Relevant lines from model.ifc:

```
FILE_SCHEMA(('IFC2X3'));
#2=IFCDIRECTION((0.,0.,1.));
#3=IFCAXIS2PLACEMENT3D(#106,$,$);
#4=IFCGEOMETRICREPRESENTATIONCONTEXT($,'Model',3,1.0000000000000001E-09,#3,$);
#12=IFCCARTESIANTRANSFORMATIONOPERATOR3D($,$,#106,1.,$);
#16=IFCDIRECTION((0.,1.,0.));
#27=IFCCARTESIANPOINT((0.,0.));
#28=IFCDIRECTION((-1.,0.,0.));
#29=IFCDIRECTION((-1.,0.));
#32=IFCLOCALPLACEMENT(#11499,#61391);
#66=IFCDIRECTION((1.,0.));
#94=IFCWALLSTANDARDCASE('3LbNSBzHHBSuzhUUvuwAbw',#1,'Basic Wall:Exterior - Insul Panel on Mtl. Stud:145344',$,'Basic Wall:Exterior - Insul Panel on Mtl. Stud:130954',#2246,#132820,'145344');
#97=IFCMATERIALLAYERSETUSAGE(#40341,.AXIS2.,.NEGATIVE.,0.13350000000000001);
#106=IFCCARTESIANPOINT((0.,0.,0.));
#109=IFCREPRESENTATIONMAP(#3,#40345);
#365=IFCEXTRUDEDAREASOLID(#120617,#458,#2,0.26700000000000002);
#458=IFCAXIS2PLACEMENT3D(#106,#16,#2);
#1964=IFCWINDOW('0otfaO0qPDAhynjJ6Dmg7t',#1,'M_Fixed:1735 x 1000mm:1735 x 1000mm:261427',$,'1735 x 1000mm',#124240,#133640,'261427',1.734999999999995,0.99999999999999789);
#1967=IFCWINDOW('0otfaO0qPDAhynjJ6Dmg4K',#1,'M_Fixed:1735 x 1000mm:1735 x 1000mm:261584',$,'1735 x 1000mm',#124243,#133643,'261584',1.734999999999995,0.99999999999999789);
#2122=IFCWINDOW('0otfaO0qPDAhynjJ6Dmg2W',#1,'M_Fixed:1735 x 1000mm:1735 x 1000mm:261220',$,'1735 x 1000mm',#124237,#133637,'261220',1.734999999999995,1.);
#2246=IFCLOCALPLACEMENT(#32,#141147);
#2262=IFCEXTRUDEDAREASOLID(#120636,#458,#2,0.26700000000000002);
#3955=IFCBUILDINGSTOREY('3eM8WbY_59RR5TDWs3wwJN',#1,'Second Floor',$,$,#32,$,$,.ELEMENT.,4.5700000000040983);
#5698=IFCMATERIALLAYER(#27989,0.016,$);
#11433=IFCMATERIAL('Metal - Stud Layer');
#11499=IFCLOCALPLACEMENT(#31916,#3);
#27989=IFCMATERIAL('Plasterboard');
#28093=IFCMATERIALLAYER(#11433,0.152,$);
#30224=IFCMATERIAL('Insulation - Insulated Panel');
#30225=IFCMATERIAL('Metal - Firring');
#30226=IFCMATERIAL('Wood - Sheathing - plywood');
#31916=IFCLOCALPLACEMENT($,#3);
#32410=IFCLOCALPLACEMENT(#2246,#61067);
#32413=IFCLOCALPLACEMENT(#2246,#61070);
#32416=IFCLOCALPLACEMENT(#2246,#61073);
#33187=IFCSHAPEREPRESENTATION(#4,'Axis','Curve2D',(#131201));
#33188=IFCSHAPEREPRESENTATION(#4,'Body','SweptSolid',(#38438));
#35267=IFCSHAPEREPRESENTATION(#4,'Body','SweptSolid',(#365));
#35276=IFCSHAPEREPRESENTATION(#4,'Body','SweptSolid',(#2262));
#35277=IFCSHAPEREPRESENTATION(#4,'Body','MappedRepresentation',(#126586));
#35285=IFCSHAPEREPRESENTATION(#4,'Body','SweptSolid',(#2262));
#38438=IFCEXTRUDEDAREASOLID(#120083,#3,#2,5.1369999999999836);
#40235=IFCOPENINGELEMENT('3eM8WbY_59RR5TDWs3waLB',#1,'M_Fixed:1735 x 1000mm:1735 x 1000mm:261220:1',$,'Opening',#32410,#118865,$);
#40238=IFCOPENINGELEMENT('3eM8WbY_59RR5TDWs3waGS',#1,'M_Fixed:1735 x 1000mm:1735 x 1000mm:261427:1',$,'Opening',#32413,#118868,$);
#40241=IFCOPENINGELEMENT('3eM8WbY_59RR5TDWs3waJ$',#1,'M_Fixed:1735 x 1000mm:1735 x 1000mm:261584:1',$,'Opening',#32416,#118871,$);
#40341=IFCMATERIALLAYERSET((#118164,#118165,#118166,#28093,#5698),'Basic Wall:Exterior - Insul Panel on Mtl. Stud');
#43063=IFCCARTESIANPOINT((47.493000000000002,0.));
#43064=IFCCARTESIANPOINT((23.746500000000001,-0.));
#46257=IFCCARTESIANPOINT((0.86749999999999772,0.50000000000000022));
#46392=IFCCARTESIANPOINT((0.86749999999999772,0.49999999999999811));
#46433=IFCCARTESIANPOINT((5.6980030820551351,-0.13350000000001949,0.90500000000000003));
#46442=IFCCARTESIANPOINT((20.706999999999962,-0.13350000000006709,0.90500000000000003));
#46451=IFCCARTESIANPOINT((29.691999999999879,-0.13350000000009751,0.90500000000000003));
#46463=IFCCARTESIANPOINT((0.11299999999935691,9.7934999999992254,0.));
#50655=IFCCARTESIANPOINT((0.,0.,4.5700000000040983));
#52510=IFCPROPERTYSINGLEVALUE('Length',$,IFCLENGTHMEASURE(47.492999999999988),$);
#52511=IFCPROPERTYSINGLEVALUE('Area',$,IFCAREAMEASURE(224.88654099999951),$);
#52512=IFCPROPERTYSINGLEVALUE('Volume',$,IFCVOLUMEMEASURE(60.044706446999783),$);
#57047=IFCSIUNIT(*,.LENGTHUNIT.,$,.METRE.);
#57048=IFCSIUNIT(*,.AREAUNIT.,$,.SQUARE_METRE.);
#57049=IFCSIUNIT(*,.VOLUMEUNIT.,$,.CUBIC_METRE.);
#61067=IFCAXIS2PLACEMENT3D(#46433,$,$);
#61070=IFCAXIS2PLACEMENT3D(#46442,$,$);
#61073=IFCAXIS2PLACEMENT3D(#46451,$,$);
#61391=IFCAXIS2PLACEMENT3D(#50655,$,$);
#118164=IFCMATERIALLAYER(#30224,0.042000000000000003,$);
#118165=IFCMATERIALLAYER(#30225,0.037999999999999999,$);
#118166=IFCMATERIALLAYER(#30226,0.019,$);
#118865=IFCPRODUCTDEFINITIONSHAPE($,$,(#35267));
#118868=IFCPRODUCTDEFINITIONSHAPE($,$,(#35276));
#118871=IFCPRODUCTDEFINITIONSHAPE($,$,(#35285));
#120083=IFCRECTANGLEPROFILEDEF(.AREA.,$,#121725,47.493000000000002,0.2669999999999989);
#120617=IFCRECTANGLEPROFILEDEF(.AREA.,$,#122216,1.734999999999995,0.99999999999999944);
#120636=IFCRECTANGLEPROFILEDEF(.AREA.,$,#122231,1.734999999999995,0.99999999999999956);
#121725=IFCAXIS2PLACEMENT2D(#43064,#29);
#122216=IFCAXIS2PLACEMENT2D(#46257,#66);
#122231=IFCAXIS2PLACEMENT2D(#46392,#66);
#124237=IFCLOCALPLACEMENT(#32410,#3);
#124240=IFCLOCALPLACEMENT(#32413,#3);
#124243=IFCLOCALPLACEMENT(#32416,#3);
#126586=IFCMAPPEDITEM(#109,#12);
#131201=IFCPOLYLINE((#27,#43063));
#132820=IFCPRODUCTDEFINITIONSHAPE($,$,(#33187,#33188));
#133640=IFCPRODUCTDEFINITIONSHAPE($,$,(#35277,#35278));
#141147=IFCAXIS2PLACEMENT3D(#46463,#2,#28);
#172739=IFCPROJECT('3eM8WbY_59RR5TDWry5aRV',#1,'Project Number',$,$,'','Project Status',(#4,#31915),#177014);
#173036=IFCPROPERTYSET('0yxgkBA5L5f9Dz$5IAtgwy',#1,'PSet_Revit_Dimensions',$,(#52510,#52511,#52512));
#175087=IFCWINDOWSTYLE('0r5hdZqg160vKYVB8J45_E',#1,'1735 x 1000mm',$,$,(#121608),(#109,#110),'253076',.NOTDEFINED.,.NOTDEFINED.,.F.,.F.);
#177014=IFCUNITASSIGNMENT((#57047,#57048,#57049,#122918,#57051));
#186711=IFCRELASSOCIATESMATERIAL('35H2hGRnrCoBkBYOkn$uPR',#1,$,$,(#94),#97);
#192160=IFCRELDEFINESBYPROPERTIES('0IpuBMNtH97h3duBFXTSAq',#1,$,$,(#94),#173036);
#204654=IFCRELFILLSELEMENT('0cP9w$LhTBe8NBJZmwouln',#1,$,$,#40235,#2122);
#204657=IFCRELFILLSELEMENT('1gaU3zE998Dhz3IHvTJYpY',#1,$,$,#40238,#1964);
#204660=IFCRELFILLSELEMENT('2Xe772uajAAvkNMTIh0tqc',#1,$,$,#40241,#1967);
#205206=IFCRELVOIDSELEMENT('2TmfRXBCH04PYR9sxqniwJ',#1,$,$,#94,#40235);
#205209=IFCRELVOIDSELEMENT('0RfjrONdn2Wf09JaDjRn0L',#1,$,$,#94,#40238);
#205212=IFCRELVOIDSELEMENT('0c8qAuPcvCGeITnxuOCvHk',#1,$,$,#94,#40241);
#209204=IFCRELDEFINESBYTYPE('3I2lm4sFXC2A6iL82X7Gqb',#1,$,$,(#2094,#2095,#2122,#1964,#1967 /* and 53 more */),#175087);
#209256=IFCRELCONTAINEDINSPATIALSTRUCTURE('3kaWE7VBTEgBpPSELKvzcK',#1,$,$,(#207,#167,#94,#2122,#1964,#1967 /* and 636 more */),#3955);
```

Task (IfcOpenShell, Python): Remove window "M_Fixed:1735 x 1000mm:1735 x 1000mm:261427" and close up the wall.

```python
import ifcopenshell
import ifcopenshell.api.feature
import ifcopenshell.api.pset
import ifcopenshell.api.root
import ifcopenshell.geom
import ifcopenshell.util.element
import ifcopenshell.util.shape
import ifcopenshell.util.unit

model = ifcopenshell.open("model.ifc")
area_scale = ifcopenshell.util.unit.calculate_unit_scale(model, "AREAUNIT")
volume_scale = ifcopenshell.util.unit.calculate_unit_scale(model, "VOLUMEUNIT")
settings = ifcopenshell.geom.settings()


def volume(element):
    """Net volume in cubic metres, openings subtracted."""
    shape = ifcopenshell.geom.create_shape(settings, element)
    return ifcopenshell.util.shape.get_volume(shape.geometry)


window = model.by_guid("0otfaO0qPDAhynjJ6Dmg7t")
opening = window.FillsVoids[0].RelatingOpeningElement
wall = opening.VoidsElements[0].RelatingBuildingElement
before = volume(wall)

ifcopenshell.api.root.remove_product(model, product=window)
ifcopenshell.api.feature.remove_feature(model, feature=opening)

after = volume(wall)
thickness = 0.267  # wall thickness in metres

# Update the wall's stored quantities.
pset = model.by_id(ifcopenshell.util.element.get_pset(wall, "PSet_Revit_Dimensions", should_inherit=False)["id"])
ifcopenshell.api.pset.edit_pset(model, pset=pset, properties={
    "Area": model.create_entity("IfcAreaMeasure", after / thickness / area_scale),
    "Volume": model.create_entity("IfcVolumeMeasure", after / volume_scale),
})

print(f"wall volume {before:.3f} -> {after:.3f} m3")

model.write("model_rev.ifc")
```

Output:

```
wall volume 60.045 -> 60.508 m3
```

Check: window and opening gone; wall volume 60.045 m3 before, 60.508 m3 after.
